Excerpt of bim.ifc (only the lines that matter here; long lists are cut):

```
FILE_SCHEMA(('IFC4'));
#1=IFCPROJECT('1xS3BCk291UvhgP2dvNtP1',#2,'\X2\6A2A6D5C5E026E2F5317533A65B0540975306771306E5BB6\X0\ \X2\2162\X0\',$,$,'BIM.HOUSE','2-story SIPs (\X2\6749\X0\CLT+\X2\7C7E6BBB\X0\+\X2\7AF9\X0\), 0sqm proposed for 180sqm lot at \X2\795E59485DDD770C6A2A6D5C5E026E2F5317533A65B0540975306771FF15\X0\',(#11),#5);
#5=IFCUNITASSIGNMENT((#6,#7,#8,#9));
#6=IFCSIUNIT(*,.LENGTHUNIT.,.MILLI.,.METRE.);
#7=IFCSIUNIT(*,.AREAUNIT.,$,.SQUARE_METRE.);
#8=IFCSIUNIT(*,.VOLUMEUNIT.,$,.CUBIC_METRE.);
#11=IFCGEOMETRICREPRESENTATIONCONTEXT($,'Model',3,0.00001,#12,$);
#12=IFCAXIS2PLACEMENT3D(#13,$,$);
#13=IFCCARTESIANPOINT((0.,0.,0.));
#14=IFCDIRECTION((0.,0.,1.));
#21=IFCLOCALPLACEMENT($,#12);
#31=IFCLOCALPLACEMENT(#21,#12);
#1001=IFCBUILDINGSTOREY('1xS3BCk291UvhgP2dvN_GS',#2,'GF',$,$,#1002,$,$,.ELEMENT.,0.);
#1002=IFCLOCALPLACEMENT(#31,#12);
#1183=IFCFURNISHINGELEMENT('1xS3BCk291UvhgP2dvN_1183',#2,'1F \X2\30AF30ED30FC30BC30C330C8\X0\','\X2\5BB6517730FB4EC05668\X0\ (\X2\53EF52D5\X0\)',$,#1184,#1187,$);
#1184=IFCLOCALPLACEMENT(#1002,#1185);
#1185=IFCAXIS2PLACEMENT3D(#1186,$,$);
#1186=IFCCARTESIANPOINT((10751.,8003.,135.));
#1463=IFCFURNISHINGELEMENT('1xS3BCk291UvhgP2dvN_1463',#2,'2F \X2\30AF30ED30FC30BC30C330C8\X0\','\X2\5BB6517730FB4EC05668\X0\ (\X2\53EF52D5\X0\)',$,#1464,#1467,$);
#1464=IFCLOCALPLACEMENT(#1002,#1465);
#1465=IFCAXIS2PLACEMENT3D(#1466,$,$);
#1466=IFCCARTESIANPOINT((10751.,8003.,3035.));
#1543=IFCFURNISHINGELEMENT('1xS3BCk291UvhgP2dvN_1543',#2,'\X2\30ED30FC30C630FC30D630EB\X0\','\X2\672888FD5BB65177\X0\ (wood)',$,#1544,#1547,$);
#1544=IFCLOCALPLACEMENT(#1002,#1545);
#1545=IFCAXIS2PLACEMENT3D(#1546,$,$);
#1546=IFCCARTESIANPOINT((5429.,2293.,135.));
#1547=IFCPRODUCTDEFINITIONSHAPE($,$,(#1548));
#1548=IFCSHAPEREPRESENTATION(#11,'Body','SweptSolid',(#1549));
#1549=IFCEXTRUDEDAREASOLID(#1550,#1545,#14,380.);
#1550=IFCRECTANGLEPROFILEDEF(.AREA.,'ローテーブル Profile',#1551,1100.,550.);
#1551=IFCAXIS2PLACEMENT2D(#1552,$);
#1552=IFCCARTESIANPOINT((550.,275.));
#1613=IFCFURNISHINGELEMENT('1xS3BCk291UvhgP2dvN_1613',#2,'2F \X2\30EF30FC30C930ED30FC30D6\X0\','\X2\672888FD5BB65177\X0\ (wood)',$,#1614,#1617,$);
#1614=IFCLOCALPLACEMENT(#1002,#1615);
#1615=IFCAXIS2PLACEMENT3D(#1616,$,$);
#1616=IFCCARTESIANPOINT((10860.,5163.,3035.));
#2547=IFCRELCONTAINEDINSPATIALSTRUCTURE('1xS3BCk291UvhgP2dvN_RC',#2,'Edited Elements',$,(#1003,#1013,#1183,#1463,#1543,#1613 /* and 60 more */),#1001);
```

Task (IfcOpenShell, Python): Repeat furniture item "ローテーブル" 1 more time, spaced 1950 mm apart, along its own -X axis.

```python
import ifcopenshell
import ifcopenshell.api.geometry
import ifcopenshell.api.root
import ifcopenshell.util.element
import ifcopenshell.util.placement
import ifcopenshell.util.unit

model = ifcopenshell.open("bim.ifc")
unit_scale = ifcopenshell.util.unit.calculate_unit_scale(model)


def reuse_history(source, copy):
    """copy_class also copies each property set's owner history, people and application; keep the originals."""
    for rel in copy.IsDefinedBy:
        if rel.is_a("IfcRelDefinesByProperties") and (history := rel.RelatingPropertyDefinition.OwnerHistory):
            rel.RelatingPropertyDefinition.OwnerHistory = source.OwnerHistory
            ifcopenshell.util.element.remove_deep2(model, history)


source = model.by_guid("1xS3BCk291UvhgP2dvN_1543")
base = ifcopenshell.util.placement.get_local_placement(source.ObjectPlacement)
step = -base[:3, 0] * 1.95 / unit_scale

for i in range(1, 2):
    copy = ifcopenshell.api.root.copy_class(model, product=source)
    copy.Representation = ifcopenshell.util.element.copy_deep(
        model, source.Representation, exclude=["IfcGeometricRepresentationContext", "IfcRepresentationMap"]
    )
    reuse_history(source, copy)
    matrix = base.copy()
    matrix[:3, 3] += i * step
    print("added at", matrix[:3, 3].round(3) + 0.0)
    ifcopenshell.api.geometry.edit_object_placement(model, product=copy, matrix=matrix, is_si=False)

model.write("bim_edited.ifc")
```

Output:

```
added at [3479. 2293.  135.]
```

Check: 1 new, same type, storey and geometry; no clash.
